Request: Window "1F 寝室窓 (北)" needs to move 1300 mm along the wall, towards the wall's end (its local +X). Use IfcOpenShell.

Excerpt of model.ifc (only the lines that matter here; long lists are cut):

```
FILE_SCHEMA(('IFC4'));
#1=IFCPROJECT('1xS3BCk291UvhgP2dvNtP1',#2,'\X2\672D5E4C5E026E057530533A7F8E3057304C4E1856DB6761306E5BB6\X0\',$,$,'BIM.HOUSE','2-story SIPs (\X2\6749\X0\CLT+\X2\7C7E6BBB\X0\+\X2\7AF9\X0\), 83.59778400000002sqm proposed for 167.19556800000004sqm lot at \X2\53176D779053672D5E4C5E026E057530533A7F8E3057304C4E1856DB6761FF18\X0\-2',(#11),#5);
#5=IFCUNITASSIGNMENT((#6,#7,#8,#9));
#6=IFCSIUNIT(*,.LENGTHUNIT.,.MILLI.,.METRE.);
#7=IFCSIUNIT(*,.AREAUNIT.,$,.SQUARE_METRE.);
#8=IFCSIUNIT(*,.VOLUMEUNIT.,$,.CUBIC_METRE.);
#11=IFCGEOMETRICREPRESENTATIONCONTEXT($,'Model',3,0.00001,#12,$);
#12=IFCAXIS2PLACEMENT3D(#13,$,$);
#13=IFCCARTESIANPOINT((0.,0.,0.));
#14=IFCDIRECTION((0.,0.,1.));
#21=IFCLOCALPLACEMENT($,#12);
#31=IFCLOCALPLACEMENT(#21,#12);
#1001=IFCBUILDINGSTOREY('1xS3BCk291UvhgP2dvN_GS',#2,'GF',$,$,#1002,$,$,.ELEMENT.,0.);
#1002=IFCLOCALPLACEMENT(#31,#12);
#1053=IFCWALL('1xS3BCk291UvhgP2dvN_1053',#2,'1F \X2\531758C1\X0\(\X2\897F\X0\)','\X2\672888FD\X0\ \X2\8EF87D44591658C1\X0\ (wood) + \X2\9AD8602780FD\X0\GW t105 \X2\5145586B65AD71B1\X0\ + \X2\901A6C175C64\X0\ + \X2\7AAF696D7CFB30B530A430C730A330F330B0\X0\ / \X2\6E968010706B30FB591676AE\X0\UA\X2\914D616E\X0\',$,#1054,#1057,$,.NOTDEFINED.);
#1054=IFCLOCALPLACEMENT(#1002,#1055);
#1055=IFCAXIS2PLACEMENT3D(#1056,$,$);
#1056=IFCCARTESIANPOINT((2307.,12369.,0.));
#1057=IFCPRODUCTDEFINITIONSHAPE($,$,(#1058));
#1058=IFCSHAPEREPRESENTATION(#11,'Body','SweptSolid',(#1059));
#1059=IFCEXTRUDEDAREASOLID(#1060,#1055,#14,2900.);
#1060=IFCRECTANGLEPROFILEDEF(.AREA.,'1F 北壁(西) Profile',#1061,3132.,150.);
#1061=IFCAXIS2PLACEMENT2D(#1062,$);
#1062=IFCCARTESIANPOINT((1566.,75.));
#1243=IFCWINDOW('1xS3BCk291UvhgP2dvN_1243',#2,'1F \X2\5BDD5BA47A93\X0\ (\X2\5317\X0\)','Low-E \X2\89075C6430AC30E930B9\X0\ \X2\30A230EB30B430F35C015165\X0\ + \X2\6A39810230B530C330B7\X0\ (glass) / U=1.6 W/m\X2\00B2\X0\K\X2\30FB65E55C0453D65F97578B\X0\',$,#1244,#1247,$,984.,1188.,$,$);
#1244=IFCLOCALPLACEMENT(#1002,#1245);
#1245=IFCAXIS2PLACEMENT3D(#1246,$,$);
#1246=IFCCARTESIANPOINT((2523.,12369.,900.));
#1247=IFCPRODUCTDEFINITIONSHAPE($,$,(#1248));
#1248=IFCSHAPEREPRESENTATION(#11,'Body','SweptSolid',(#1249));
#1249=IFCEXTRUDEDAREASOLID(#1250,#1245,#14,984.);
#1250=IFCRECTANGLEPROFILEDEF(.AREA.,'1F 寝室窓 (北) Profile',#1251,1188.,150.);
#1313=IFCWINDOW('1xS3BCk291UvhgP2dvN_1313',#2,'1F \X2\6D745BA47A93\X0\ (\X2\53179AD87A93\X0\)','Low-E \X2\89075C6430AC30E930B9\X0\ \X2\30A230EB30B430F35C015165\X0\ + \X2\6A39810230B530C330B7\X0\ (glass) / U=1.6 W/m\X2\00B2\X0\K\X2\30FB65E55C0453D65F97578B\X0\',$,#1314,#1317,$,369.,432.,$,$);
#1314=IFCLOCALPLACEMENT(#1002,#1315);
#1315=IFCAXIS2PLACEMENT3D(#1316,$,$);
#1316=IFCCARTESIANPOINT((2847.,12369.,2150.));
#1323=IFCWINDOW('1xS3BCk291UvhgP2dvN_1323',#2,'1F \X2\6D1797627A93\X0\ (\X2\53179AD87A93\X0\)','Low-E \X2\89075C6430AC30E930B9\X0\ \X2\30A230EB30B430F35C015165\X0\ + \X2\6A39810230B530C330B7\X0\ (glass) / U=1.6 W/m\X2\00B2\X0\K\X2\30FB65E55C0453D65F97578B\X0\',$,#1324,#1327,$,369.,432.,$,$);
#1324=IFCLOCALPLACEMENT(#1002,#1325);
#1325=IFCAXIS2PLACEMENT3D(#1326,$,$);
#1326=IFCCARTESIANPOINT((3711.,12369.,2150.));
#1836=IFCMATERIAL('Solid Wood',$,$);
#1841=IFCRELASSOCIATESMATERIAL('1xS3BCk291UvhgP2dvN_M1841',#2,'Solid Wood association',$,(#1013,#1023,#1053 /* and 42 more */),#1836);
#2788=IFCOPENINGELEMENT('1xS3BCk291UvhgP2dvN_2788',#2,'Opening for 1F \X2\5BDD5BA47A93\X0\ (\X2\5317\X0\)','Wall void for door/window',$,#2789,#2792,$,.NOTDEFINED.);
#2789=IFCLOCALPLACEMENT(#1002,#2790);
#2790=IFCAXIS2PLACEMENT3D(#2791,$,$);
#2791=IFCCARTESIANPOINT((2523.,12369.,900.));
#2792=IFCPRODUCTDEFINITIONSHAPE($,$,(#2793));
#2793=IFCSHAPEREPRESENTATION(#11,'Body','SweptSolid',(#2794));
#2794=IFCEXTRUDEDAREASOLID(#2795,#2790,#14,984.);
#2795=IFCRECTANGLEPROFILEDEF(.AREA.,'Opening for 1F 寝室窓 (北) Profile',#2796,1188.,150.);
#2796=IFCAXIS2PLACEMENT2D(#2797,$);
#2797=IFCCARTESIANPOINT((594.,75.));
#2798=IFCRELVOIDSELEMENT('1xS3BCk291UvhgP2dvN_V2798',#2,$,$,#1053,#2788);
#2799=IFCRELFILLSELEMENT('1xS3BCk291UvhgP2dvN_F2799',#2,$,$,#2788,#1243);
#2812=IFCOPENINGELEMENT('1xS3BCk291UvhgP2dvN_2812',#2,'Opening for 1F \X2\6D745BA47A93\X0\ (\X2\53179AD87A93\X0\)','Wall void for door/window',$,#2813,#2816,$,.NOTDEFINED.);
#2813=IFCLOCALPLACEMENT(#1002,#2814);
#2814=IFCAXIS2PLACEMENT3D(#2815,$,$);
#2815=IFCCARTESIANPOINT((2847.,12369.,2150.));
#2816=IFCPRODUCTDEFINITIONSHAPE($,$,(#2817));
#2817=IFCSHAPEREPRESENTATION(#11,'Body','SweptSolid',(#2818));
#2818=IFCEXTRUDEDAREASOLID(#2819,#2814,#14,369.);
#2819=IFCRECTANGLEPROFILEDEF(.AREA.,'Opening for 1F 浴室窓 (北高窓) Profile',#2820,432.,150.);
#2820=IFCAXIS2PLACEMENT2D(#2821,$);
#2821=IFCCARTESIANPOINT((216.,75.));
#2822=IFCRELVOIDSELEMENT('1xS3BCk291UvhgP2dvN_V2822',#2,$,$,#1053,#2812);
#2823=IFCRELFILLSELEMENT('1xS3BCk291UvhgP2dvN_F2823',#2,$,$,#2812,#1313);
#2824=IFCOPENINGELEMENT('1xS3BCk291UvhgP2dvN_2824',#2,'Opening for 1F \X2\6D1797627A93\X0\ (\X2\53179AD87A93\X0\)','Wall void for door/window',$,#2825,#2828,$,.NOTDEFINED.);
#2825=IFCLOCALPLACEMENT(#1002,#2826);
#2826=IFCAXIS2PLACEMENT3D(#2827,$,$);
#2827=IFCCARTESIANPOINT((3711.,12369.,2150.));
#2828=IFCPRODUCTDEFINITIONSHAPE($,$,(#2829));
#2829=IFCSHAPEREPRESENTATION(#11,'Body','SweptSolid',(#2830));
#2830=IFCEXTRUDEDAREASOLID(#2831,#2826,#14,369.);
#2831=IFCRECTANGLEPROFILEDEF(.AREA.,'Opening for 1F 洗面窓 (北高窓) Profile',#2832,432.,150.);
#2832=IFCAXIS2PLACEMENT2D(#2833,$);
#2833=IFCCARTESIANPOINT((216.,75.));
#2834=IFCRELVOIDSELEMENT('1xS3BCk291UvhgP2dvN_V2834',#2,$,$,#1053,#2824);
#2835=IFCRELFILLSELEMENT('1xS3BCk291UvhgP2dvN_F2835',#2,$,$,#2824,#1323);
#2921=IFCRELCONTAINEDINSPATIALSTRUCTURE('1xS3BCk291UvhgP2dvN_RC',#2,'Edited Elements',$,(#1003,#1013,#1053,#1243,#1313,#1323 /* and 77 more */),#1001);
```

```python
import ifcopenshell
import ifcopenshell.api.geometry
import ifcopenshell.util.placement
import ifcopenshell.util.unit

model = ifcopenshell.open("model.ifc")
unit_scale = ifcopenshell.util.unit.calculate_unit_scale(model)

window = model.by_guid("1xS3BCk291UvhgP2dvN_1243")
opening = window.FillsVoids[0].RelatingOpeningElement
wall = opening.VoidsElements[0].RelatingBuildingElement

wall_matrix = ifcopenshell.util.placement.get_local_placement(wall.ObjectPlacement)
shift = wall_matrix[:3, 0] * 1.3 / unit_scale
before = ifcopenshell.util.placement.get_local_placement(window.ObjectPlacement)[:3, 3].copy()

# The window is not placed relative to its opening, so move both.
for product in (opening, window):
    matrix = ifcopenshell.util.placement.get_local_placement(product.ObjectPlacement)
    matrix[:3, 3] += shift
    ifcopenshell.api.geometry.edit_object_placement(model, product=product, matrix=matrix, is_si=False)

after = ifcopenshell.util.placement.get_local_placement(window.ObjectPlacement)[:3, 3]
print("window moved by", (after - before).round(3) + 0.0)

model.write("model_edited.ifc")
```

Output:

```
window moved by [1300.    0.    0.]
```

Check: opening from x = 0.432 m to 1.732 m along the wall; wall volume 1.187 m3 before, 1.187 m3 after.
